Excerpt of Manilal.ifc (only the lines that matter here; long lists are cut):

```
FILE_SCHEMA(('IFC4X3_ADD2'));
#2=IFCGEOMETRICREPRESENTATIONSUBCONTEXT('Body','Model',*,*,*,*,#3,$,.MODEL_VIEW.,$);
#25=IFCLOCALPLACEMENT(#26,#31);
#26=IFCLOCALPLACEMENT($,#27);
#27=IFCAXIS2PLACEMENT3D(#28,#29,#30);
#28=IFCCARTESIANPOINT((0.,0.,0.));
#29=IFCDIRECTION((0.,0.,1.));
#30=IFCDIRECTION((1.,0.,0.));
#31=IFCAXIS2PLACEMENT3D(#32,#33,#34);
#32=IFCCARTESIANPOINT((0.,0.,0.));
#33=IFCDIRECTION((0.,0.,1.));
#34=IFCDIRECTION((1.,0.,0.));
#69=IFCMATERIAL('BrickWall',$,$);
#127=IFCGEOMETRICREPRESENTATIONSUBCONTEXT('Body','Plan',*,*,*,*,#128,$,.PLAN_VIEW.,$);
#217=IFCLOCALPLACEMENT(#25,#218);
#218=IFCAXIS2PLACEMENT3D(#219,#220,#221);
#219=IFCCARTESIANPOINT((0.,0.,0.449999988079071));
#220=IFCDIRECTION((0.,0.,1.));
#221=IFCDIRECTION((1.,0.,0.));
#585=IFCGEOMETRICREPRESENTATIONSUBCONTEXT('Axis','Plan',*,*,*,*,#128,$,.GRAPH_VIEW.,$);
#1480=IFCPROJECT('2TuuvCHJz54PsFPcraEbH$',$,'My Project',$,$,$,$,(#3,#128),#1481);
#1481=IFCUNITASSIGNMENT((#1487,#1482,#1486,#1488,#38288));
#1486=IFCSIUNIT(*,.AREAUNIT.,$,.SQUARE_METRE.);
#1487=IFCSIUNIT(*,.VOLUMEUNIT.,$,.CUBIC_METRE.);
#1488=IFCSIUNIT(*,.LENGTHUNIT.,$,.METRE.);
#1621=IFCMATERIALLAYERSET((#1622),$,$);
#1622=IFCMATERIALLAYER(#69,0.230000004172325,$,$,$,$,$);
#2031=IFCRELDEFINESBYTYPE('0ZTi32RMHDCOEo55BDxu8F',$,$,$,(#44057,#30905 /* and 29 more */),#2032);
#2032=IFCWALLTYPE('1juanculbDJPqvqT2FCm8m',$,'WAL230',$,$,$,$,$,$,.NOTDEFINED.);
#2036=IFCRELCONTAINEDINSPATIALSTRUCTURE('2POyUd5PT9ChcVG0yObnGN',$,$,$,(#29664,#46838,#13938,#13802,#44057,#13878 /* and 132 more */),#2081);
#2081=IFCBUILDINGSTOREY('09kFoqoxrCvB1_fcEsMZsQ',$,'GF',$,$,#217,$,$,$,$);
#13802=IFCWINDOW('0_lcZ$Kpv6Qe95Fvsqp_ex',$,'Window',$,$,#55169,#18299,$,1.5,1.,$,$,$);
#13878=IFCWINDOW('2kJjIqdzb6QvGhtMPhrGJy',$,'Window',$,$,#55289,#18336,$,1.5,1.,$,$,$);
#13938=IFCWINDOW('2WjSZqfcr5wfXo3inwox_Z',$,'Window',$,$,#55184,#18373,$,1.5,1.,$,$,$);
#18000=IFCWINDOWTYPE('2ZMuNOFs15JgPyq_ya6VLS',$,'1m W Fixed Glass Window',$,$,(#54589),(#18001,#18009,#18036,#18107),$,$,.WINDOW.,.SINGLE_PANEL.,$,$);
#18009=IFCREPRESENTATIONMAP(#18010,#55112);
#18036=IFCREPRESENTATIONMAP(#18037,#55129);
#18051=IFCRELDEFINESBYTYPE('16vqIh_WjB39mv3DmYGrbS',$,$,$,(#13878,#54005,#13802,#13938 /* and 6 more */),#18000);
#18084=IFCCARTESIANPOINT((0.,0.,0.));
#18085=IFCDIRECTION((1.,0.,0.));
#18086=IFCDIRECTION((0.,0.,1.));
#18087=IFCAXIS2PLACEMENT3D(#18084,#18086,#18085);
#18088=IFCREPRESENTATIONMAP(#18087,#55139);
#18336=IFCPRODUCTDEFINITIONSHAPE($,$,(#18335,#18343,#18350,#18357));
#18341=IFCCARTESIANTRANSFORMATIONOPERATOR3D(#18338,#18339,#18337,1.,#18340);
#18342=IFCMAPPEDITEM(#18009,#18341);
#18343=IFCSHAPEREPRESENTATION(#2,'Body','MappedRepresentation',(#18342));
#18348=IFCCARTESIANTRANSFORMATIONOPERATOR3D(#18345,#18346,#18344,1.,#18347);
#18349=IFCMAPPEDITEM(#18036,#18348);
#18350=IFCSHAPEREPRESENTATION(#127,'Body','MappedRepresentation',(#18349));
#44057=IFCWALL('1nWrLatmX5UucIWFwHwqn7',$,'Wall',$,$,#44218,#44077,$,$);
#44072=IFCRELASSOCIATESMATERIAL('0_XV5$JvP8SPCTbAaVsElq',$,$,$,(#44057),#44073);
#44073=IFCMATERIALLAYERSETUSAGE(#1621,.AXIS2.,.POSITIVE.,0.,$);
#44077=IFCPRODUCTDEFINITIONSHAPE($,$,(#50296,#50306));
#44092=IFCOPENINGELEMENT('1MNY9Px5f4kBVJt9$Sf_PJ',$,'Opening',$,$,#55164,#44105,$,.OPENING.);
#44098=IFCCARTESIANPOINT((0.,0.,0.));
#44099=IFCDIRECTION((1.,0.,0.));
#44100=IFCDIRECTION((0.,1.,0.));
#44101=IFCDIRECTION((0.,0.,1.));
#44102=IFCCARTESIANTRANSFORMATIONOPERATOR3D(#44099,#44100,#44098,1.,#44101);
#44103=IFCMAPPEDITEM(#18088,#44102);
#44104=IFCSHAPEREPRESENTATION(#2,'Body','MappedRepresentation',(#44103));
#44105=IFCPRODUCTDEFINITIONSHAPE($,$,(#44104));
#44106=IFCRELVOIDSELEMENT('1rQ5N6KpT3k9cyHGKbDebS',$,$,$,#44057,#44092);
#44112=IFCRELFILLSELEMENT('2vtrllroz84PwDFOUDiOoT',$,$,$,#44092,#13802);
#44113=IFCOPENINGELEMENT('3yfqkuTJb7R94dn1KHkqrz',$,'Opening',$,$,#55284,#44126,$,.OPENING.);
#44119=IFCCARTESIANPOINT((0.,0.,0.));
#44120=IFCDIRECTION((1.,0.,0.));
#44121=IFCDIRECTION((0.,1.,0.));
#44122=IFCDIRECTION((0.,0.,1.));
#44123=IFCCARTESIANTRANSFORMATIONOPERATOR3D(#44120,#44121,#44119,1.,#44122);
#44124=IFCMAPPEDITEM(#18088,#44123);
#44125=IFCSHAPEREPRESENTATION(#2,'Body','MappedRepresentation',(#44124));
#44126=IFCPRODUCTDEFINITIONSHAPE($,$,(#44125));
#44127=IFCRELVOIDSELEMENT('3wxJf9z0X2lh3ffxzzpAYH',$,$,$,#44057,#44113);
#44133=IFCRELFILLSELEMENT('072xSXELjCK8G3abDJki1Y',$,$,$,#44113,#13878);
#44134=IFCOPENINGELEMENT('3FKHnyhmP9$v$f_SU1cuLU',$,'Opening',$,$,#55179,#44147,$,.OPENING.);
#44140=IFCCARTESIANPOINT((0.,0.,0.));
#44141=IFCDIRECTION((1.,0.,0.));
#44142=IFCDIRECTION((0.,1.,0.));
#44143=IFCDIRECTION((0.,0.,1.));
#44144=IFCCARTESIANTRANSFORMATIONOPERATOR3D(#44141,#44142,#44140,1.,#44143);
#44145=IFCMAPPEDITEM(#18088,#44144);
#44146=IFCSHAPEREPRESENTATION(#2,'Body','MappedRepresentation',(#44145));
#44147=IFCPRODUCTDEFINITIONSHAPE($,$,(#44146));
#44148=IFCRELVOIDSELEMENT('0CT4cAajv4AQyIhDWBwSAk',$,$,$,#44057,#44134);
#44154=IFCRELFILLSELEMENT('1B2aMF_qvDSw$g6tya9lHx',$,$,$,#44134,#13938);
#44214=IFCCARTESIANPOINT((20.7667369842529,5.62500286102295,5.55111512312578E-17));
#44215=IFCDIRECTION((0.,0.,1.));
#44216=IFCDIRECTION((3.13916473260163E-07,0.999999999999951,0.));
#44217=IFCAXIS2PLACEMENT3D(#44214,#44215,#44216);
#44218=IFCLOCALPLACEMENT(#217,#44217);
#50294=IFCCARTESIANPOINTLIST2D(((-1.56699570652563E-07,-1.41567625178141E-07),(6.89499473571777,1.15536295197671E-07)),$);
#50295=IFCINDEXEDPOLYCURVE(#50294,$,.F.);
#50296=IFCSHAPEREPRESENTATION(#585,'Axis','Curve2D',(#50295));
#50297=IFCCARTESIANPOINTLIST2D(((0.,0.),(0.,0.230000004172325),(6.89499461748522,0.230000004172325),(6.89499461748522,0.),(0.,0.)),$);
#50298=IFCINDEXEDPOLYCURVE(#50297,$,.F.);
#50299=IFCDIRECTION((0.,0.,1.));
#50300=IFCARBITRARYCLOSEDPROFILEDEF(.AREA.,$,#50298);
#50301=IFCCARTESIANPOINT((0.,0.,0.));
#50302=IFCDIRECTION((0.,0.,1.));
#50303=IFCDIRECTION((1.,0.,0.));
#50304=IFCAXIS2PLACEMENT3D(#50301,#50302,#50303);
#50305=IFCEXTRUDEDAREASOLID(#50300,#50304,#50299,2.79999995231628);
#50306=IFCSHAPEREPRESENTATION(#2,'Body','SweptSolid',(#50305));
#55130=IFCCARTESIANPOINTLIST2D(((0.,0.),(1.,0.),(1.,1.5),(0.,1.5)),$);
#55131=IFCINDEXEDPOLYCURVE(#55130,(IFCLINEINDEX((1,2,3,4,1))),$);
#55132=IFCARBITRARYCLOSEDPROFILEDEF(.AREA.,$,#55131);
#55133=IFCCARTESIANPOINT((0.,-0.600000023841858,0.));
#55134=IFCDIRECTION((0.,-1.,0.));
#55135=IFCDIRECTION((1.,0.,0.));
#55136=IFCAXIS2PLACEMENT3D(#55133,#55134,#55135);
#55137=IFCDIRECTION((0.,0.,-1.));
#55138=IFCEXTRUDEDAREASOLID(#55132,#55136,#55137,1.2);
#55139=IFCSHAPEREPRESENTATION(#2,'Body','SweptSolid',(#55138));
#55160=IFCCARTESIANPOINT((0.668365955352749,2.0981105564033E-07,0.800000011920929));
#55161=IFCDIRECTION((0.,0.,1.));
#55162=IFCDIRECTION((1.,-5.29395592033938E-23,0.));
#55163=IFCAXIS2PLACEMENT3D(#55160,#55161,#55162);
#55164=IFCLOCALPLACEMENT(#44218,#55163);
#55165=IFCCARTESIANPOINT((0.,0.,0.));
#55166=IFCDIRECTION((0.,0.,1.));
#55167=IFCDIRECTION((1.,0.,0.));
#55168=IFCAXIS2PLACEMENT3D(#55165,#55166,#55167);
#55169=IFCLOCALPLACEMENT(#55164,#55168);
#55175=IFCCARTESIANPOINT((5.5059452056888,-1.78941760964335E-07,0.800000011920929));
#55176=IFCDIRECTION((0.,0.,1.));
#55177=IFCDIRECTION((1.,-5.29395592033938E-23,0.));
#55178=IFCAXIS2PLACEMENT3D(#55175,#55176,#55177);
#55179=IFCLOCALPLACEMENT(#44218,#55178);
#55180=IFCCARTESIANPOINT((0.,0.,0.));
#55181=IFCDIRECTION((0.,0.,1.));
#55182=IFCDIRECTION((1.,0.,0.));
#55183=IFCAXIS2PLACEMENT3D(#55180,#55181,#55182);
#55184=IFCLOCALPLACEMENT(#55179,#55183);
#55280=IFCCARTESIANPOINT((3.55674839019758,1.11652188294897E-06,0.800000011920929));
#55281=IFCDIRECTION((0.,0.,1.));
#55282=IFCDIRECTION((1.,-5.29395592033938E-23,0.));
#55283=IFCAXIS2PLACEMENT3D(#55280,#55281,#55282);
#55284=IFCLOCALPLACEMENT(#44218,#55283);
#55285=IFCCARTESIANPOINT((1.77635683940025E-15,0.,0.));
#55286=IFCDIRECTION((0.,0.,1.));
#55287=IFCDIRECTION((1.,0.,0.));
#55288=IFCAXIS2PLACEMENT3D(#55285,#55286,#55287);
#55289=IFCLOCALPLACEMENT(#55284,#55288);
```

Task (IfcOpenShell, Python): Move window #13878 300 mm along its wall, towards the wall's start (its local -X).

```python
import ifcopenshell
import ifcopenshell.api.geometry
import ifcopenshell.util.placement
import ifcopenshell.util.unit

model = ifcopenshell.open("Manilal.ifc")
unit_scale = ifcopenshell.util.unit.calculate_unit_scale(model)

window = model.by_id(13878)
opening = window.FillsVoids[0].RelatingOpeningElement
wall = opening.VoidsElements[0].RelatingBuildingElement

wall_matrix = ifcopenshell.util.placement.get_local_placement(wall.ObjectPlacement)
shift = wall_matrix[:3, 0] * -0.3 / unit_scale
before = ifcopenshell.util.placement.get_local_placement(window.ObjectPlacement)[:3, 3].copy()

# The window is placed relative to its opening, so it follows when the opening moves.
matrix = ifcopenshell.util.placement.get_local_placement(opening.ObjectPlacement)
matrix[:3, 3] += shift
ifcopenshell.api.geometry.edit_object_placement(
    model, product=opening, matrix=matrix, is_si=False, should_transform_children=True
)

after = ifcopenshell.util.placement.get_local_placement(window.ObjectPlacement)[:3, 3]
print("window moved by", (after - before).round(3) + 0.0)

model.write("Manilal_updated.ifc")
```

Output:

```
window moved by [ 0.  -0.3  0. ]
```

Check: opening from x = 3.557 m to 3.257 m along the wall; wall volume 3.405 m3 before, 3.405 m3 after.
